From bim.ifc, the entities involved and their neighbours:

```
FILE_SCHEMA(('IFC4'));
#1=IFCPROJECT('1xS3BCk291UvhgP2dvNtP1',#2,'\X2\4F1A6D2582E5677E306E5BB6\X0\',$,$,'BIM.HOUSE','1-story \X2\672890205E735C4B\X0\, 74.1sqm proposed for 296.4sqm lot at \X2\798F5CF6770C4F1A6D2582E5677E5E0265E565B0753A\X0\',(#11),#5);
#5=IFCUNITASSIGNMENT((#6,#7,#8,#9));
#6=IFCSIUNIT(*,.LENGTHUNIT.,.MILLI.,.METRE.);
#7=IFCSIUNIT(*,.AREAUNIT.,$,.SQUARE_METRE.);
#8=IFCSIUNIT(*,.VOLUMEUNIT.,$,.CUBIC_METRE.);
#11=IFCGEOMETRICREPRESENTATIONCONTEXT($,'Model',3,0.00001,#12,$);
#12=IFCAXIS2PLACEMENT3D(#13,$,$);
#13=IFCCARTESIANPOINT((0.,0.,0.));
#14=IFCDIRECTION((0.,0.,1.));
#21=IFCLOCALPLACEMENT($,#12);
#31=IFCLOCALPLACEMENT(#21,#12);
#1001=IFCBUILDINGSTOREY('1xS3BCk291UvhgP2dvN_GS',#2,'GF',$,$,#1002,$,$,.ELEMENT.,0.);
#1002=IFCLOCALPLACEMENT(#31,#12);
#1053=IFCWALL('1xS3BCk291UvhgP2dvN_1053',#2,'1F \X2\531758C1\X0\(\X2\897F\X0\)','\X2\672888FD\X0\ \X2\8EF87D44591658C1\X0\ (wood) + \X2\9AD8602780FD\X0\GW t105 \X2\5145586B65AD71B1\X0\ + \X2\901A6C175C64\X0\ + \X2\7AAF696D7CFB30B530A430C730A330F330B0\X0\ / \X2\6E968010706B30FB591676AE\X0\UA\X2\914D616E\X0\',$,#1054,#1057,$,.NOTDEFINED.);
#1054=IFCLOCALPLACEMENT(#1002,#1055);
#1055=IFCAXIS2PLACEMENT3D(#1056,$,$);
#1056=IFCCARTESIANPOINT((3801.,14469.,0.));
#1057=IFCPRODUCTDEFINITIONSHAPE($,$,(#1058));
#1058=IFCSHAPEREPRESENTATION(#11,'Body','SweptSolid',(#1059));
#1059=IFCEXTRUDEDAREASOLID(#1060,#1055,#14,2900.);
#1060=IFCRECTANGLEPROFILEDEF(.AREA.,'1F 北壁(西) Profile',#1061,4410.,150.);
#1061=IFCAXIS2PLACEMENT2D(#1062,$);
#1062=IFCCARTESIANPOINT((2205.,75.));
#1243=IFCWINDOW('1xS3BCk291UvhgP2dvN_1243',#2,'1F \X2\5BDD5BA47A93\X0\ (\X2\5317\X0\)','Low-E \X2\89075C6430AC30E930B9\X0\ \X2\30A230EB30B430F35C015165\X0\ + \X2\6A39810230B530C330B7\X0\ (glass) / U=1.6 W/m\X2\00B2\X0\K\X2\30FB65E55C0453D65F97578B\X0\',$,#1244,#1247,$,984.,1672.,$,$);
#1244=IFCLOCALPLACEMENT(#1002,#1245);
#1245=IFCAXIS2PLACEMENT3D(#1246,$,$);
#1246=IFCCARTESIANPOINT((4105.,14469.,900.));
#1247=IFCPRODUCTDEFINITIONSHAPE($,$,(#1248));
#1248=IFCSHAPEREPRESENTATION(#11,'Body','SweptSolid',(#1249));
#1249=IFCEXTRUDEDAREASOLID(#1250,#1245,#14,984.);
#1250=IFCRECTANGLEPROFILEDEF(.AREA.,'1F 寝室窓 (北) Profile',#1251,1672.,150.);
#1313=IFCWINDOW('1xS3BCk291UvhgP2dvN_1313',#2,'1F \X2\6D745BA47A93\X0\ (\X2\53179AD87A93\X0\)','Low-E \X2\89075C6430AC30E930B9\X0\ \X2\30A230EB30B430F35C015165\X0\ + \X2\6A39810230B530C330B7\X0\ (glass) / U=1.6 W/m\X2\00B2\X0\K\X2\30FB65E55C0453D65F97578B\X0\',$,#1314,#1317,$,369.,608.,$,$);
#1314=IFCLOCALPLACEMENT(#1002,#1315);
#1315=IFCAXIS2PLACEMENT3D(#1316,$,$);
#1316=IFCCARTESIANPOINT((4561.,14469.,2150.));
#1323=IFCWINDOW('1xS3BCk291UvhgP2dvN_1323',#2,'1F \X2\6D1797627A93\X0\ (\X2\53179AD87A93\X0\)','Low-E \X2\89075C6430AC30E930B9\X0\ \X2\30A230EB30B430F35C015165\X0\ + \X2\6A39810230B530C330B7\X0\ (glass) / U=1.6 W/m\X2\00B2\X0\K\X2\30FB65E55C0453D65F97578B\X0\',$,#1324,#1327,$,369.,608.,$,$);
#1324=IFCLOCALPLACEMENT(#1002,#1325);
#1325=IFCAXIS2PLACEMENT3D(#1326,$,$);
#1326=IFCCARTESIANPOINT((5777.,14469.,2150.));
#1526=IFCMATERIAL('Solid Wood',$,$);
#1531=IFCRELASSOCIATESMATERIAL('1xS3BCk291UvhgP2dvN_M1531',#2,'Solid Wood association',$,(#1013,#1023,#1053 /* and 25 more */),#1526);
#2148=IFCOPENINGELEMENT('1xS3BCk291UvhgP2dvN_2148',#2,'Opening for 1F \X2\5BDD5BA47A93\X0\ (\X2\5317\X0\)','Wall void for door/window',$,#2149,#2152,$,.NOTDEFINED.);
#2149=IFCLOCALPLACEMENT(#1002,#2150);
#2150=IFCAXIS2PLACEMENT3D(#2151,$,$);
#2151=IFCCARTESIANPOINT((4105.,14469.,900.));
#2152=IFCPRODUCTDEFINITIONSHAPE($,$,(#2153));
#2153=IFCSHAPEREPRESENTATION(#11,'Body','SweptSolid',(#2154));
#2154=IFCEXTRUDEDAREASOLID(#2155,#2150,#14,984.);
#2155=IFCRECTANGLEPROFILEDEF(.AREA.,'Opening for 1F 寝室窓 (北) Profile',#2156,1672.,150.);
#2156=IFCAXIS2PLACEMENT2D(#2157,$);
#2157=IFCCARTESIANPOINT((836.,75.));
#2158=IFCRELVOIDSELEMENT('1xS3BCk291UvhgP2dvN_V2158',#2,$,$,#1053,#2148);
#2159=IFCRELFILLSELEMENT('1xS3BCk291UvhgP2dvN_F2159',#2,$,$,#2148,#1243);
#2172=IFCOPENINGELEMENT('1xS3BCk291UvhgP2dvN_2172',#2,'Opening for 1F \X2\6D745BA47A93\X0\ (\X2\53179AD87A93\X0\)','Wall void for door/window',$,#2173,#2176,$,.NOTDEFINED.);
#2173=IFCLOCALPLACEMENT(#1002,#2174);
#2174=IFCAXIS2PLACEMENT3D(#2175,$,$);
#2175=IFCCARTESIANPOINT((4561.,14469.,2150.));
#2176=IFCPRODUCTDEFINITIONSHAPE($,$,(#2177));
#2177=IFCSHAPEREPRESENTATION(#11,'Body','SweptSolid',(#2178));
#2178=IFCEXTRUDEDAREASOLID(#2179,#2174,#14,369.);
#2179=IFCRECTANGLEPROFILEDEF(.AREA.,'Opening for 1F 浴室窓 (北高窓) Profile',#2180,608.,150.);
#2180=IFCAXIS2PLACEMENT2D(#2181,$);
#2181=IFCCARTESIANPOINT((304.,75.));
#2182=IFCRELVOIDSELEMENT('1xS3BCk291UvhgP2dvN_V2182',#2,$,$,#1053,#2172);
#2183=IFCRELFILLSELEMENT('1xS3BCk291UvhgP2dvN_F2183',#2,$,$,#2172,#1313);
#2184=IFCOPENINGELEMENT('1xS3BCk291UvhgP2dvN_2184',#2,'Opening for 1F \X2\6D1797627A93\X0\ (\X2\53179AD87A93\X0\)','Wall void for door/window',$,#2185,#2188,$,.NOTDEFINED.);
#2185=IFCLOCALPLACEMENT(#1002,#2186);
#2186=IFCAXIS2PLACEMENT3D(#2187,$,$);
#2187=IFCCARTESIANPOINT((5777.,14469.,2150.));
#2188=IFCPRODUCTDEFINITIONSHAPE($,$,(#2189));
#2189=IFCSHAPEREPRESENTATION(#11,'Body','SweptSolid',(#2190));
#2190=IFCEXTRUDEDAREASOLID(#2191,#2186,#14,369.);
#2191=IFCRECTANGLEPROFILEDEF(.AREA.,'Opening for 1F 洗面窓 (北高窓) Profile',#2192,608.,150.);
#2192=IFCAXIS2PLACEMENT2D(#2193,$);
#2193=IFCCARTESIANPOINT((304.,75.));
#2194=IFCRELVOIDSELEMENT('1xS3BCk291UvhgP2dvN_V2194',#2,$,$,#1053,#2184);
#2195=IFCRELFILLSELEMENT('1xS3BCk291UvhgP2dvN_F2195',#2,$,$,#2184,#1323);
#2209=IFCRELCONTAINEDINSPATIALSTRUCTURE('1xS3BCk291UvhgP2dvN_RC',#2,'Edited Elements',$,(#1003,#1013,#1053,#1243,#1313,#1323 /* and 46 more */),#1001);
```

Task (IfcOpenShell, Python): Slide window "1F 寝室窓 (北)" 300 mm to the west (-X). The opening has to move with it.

```python
import ifcopenshell
import ifcopenshell.api.geometry
import ifcopenshell.util.placement
import ifcopenshell.util.unit

model = ifcopenshell.open("bim.ifc")
unit_scale = ifcopenshell.util.unit.calculate_unit_scale(model)

window = model.by_guid("1xS3BCk291UvhgP2dvN_1243")
opening = window.FillsVoids[0].RelatingOpeningElement
wall = opening.VoidsElements[0].RelatingBuildingElement

wall_matrix = ifcopenshell.util.placement.get_local_placement(wall.ObjectPlacement)
shift = wall_matrix[:3, 0] * -0.3 / unit_scale
before = ifcopenshell.util.placement.get_local_placement(window.ObjectPlacement)[:3, 3].copy()

# The window is not placed relative to its opening, so move both.
for product in (opening, window):
    matrix = ifcopenshell.util.placement.get_local_placement(product.ObjectPlacement)
    matrix[:3, 3] += shift
    ifcopenshell.api.geometry.edit_object_placement(model, product=product, matrix=matrix, is_si=False)

after = ifcopenshell.util.placement.get_local_placement(window.ObjectPlacement)[:3, 3]
print("window moved by", (after - before).round(3) + 0.0)

model.write("bim_updated.ifc")
```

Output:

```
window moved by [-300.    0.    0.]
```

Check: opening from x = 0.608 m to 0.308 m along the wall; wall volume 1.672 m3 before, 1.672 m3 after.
